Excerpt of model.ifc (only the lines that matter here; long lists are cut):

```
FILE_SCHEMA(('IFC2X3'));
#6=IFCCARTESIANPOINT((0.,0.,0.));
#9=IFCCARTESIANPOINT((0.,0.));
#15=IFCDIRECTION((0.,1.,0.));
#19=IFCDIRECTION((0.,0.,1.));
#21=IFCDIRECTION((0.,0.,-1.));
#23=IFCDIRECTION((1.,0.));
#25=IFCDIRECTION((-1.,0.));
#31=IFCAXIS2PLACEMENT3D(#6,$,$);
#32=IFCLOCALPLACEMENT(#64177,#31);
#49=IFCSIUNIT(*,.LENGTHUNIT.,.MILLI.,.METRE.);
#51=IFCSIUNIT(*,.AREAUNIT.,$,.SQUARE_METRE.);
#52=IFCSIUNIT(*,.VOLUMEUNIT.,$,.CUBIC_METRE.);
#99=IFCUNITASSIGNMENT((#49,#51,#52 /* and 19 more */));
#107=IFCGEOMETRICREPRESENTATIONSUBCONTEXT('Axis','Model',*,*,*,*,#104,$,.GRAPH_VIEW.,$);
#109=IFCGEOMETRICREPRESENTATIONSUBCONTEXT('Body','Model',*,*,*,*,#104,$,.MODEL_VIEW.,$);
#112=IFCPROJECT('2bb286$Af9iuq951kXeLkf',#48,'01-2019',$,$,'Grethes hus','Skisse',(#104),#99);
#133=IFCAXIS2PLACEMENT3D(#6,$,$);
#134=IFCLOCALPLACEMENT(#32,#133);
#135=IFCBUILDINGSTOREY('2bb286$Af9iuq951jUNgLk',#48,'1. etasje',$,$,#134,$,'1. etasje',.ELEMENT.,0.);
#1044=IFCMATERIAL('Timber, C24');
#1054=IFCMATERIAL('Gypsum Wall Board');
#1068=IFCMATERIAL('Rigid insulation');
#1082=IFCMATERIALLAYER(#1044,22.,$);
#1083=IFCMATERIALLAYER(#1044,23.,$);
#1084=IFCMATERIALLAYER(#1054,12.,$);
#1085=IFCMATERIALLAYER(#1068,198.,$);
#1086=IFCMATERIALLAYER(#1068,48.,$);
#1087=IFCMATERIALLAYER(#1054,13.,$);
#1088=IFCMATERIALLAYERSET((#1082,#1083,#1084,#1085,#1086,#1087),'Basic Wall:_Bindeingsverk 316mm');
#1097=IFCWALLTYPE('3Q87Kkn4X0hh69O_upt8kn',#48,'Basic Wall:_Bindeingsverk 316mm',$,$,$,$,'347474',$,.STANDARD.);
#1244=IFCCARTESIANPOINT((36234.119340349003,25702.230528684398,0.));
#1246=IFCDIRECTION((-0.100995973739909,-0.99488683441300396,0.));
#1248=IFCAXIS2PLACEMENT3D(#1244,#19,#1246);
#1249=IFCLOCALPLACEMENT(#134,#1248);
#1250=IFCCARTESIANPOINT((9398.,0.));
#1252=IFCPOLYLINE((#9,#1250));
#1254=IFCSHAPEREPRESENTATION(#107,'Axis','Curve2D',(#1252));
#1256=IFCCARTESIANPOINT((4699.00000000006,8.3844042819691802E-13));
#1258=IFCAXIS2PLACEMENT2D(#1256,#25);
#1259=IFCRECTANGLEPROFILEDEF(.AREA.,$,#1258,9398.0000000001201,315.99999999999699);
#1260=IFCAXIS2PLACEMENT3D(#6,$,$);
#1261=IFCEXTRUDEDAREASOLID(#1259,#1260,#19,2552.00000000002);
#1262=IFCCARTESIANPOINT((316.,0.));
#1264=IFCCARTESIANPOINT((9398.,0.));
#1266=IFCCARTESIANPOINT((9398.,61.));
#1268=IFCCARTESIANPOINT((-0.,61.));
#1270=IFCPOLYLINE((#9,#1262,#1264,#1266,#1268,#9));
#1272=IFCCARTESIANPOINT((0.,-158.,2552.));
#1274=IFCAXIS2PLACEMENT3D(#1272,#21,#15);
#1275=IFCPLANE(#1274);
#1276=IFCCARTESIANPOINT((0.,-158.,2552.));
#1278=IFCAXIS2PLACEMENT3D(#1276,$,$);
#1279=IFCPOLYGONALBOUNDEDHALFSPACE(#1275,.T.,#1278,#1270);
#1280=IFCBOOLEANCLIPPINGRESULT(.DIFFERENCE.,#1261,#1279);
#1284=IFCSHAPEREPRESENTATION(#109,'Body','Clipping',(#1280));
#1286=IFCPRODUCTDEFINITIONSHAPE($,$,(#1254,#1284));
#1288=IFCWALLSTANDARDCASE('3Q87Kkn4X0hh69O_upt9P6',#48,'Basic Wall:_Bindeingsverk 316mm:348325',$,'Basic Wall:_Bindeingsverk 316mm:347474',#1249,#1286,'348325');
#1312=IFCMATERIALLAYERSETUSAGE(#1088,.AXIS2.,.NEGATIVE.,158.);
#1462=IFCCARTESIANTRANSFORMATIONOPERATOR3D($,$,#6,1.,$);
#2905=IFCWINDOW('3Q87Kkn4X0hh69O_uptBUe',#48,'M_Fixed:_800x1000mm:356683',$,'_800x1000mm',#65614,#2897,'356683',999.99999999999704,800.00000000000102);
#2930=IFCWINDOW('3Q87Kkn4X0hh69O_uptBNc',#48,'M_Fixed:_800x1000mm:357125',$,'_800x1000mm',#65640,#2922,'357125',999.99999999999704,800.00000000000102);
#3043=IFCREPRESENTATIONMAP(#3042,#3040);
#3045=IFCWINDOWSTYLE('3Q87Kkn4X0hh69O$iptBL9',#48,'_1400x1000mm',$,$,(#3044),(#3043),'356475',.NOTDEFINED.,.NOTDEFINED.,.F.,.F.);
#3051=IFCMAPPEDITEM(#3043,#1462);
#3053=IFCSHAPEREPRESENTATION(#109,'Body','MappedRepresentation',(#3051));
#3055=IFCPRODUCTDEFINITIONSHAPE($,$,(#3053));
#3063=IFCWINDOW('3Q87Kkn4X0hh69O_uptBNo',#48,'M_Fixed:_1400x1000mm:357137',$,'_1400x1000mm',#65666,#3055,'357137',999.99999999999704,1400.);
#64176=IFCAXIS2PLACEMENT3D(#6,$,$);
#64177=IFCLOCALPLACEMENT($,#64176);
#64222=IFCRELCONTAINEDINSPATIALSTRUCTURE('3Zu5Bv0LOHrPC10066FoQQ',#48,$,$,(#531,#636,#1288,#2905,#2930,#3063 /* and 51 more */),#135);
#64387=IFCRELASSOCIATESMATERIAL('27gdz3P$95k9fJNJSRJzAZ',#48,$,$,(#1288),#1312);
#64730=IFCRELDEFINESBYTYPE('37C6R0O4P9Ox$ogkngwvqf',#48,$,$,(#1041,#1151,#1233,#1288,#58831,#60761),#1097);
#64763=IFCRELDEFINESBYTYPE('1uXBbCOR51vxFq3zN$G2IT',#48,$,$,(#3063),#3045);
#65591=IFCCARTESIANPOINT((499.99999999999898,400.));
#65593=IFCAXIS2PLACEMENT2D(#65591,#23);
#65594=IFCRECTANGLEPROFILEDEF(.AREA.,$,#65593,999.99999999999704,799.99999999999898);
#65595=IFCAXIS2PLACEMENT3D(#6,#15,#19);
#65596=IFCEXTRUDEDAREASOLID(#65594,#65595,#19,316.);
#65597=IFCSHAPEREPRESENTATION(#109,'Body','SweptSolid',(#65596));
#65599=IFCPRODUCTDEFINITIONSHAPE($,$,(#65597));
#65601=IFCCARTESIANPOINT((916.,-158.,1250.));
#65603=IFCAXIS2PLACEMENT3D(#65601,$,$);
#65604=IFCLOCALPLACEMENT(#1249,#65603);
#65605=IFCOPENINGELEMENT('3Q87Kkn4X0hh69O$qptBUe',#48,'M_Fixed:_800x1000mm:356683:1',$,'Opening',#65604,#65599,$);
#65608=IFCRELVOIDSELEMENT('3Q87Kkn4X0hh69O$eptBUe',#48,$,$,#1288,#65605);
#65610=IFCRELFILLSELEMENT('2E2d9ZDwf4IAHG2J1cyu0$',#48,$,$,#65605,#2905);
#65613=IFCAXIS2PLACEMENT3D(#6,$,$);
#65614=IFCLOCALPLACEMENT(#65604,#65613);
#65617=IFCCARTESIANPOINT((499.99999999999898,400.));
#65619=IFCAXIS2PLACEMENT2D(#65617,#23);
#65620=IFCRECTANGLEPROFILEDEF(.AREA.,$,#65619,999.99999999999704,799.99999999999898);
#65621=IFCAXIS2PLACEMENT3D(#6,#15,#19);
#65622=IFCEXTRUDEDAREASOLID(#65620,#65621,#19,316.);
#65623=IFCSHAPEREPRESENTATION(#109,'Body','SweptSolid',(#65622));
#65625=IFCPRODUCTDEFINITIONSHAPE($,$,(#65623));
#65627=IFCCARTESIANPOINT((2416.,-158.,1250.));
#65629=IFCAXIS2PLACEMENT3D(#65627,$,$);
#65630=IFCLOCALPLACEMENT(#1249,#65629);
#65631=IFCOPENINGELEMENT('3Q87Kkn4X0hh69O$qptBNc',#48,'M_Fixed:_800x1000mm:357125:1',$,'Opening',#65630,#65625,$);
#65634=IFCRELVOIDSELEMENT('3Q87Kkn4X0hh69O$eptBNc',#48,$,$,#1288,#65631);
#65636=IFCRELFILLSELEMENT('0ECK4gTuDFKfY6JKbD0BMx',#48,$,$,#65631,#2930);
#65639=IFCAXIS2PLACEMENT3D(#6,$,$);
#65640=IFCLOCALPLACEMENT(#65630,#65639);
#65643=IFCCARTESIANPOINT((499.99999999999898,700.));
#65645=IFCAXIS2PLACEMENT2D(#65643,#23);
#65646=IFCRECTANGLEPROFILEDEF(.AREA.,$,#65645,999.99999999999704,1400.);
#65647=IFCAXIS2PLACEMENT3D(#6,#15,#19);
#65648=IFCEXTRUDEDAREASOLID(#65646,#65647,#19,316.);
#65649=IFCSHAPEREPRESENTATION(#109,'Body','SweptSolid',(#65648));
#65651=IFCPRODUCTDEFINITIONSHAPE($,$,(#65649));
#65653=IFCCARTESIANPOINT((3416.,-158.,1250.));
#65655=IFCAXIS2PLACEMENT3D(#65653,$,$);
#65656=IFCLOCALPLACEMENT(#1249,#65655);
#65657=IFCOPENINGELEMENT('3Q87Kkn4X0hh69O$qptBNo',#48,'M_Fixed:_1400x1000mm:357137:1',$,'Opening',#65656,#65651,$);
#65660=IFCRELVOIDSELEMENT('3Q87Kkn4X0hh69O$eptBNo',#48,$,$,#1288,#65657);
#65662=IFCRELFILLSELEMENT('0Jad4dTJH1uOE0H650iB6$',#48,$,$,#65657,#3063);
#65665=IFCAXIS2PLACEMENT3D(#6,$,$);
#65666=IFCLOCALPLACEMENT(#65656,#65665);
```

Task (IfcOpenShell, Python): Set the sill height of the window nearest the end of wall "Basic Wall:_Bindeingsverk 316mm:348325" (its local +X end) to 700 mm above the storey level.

```python
import numpy as np
import ifcopenshell
import ifcopenshell.api.geometry
import ifcopenshell.geom
import ifcopenshell.util.element
import ifcopenshell.util.placement
import ifcopenshell.util.shape
import ifcopenshell.util.unit

model = ifcopenshell.open("model.ifc")
unit_scale = ifcopenshell.util.unit.calculate_unit_scale(model)

window = model.by_guid("3Q87Kkn4X0hh69O_uptBNo")
opening = window.FillsVoids[0].RelatingOpeningElement
storey = ifcopenshell.util.element.get_container(window, ifc_class="IfcBuildingStorey")
level = ifcopenshell.util.placement.get_local_placement(storey.ObjectPlacement)[2, 3]

# The opening's origin need not be at the sill, so measure its lowest point.
shape = ifcopenshell.geom.create_shape(ifcopenshell.geom.settings(), opening)
bottom = ifcopenshell.util.shape.get_shape_bottom_elevation(shape, shape.geometry) / unit_scale
dz = level + 0.7 / unit_scale - bottom

shift = np.array([0.0, 0.0, dz])
# The window is placed relative to its opening, so it follows when the opening moves.
matrix = ifcopenshell.util.placement.get_local_placement(opening.ObjectPlacement)
matrix[:3, 3] += shift
ifcopenshell.api.geometry.edit_object_placement(
    model, product=opening, matrix=matrix, is_si=False, should_transform_children=True
)

print(f"moved by {dz * unit_scale:+.3f} m")

model.write("model-out.ifc")
```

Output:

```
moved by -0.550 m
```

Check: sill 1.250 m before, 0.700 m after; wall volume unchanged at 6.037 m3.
